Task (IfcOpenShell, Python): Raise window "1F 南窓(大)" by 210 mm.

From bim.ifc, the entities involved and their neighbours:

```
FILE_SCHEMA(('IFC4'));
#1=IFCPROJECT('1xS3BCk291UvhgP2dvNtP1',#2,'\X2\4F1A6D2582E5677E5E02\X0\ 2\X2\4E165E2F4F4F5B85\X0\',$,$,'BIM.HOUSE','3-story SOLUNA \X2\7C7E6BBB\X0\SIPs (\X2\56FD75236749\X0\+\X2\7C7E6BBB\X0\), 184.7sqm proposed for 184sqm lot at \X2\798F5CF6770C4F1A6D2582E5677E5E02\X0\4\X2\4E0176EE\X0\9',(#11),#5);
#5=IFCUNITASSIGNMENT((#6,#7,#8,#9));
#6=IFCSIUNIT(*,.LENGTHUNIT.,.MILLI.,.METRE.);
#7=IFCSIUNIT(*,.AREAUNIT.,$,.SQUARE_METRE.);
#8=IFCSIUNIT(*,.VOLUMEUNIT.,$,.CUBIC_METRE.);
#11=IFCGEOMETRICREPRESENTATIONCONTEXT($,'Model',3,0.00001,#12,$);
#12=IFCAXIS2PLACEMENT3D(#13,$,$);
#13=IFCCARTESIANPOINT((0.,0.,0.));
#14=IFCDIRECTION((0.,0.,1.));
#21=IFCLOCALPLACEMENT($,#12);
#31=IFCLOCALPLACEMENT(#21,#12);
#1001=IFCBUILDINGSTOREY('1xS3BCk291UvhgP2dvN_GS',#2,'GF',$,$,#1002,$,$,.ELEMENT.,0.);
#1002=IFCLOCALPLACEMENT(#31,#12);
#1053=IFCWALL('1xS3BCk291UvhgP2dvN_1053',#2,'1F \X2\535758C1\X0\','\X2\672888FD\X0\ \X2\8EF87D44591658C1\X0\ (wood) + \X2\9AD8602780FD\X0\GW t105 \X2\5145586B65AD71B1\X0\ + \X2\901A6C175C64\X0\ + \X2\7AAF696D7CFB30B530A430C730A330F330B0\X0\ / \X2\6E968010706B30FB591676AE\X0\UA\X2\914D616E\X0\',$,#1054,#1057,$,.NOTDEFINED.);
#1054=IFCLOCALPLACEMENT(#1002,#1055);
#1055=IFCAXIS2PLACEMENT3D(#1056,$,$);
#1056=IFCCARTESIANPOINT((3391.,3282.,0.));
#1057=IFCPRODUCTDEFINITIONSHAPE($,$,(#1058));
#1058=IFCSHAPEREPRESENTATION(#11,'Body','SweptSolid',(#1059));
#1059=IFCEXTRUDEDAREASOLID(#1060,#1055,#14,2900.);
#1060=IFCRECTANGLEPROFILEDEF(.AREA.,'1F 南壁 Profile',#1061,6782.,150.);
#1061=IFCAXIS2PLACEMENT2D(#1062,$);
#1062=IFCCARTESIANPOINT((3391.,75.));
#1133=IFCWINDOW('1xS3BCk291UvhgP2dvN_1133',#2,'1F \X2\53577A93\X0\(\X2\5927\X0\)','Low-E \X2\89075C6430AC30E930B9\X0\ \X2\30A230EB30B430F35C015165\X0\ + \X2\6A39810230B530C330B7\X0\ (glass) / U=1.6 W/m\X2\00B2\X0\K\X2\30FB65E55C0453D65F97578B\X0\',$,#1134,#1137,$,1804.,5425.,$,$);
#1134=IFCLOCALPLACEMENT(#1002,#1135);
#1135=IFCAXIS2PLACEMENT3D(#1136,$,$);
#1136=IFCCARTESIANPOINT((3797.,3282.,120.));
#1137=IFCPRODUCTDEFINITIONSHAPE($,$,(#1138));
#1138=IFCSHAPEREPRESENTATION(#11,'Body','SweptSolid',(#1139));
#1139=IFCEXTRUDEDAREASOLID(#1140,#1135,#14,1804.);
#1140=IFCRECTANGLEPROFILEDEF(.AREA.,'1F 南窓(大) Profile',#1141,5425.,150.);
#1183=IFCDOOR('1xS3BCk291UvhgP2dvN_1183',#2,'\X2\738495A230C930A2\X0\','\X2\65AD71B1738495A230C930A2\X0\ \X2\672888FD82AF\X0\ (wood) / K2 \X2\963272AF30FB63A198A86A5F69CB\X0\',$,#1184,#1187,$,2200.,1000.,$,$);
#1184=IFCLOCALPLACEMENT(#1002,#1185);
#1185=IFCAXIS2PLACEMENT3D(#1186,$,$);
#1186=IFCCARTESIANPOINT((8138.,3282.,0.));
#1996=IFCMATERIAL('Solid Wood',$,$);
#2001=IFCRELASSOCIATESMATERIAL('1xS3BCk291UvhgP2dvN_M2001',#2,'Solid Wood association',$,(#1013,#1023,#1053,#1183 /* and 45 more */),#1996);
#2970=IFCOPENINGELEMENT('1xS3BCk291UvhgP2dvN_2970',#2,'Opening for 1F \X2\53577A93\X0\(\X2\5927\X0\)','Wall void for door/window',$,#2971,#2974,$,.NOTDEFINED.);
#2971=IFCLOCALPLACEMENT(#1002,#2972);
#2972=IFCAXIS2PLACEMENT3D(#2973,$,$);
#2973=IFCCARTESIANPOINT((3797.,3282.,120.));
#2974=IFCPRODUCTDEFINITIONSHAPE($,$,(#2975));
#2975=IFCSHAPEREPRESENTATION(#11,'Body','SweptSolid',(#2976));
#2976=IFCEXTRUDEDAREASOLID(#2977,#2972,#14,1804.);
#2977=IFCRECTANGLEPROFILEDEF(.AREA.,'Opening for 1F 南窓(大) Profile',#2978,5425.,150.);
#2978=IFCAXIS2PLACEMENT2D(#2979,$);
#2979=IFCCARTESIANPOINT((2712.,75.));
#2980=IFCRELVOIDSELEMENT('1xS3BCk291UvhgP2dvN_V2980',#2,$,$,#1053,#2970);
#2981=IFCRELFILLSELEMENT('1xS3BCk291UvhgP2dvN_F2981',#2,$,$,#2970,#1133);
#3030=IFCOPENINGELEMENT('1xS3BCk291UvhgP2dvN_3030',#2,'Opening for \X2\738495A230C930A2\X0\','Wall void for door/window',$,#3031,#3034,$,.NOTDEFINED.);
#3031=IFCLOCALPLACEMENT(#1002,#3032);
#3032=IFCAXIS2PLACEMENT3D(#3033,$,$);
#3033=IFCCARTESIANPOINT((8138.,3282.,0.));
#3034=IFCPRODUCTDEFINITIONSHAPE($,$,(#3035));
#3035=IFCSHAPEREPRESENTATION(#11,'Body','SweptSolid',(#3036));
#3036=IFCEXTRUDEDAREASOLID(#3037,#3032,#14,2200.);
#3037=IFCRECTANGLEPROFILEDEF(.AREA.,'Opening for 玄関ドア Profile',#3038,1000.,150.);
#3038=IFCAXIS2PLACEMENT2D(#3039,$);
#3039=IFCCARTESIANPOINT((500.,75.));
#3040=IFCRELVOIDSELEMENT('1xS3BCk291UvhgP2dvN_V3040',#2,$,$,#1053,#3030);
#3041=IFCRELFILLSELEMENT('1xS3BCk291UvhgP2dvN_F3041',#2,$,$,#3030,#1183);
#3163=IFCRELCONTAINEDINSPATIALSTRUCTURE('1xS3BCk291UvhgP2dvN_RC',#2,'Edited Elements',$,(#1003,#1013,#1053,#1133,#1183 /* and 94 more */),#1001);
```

```python
import numpy as np
import ifcopenshell
import ifcopenshell.api.geometry
import ifcopenshell.util.placement
import ifcopenshell.util.unit

model = ifcopenshell.open("bim.ifc")
unit_scale = ifcopenshell.util.unit.calculate_unit_scale(model)

window = model.by_id(1133)
opening = window.FillsVoids[0].RelatingOpeningElement
dz = 210.0

shift = np.array([0.0, 0.0, dz])
# The window is not placed relative to its opening, so move both.
for product in (opening, window):
    matrix = ifcopenshell.util.placement.get_local_placement(product.ObjectPlacement)
    matrix[:3, 3] += shift
    ifcopenshell.api.geometry.edit_object_placement(model, product=product, matrix=matrix, is_si=False)

print(f"moved by {dz * unit_scale:+.3f} m")

model.write("bim-out.ifc")
```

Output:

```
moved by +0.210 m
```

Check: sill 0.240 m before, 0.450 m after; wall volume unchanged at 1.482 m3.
